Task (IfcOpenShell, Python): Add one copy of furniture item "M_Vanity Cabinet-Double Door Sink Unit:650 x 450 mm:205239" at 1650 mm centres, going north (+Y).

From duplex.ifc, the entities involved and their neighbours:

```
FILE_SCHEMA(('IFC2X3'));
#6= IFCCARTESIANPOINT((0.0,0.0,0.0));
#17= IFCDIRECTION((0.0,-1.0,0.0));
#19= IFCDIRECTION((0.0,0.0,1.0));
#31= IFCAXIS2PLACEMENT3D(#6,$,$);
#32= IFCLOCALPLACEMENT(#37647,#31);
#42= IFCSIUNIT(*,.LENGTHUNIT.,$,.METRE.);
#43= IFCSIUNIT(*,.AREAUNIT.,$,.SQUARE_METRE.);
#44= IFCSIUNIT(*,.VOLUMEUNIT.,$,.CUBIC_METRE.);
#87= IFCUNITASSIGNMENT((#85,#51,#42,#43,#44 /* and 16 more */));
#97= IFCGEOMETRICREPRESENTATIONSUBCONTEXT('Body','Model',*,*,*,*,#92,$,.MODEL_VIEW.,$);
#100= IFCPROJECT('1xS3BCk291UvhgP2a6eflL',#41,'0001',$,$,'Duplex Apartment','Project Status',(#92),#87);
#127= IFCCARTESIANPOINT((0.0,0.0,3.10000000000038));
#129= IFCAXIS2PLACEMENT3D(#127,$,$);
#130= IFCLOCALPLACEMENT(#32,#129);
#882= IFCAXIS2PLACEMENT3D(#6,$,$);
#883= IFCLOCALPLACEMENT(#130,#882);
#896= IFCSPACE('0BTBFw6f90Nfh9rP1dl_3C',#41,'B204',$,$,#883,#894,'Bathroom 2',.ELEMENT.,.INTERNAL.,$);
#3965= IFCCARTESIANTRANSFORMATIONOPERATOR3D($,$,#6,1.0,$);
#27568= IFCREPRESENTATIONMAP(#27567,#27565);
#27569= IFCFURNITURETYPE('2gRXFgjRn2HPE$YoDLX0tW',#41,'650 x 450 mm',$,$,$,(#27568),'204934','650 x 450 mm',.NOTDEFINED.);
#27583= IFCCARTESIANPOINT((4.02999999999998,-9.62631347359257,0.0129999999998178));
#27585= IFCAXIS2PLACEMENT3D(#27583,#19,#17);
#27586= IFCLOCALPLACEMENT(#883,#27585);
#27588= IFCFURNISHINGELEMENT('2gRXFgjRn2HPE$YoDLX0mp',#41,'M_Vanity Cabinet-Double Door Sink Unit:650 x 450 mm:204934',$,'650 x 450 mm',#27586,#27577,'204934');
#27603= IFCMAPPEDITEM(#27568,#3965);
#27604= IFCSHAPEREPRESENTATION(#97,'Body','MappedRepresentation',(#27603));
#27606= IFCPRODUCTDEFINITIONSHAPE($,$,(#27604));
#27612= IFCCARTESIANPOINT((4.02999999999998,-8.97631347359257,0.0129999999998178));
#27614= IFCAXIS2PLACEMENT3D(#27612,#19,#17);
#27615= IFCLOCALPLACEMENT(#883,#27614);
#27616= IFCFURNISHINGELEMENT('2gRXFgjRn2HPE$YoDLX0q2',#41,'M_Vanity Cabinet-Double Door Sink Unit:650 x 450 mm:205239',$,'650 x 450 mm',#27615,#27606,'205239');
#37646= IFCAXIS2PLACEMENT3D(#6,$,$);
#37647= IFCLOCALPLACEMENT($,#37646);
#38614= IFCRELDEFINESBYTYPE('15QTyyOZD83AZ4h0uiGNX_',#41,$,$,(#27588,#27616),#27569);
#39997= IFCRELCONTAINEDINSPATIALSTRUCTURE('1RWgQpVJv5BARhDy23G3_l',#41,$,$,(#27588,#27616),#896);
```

```python
import numpy as np
import ifcopenshell
import ifcopenshell.api.geometry
import ifcopenshell.api.root
import ifcopenshell.util.element
import ifcopenshell.util.placement
import ifcopenshell.util.unit

model = ifcopenshell.open("duplex.ifc")
unit_scale = ifcopenshell.util.unit.calculate_unit_scale(model)


def reuse_history(source, copy):
    """copy_class also copies each property set's owner history, people and application; keep the originals."""
    for rel in copy.IsDefinedBy:
        if rel.is_a("IfcRelDefinesByProperties") and (history := rel.RelatingPropertyDefinition.OwnerHistory):
            rel.RelatingPropertyDefinition.OwnerHistory = source.OwnerHistory
            ifcopenshell.util.element.remove_deep2(model, history)


source = model.by_guid("2gRXFgjRn2HPE$YoDLX0q2")
base = ifcopenshell.util.placement.get_local_placement(source.ObjectPlacement)
step = np.array([0.0, 1.0, 0.0]) * 1.65 / unit_scale

for i in range(1, 2):
    copy = ifcopenshell.api.root.copy_class(model, product=source)
    copy.Representation = ifcopenshell.util.element.copy_deep(
        model, source.Representation, exclude=["IfcGeometricRepresentationContext", "IfcRepresentationMap"]
    )
    copy.Name = "M_Vanity Cabinet-Double Door Sink Unit:650 x 450 mm"
    copy.Tag = None
    reuse_history(source, copy)
    matrix = base.copy()
    matrix[:3, 3] += i * step
    print("added at", matrix[:3, 3].round(3) + 0.0)
    ifcopenshell.api.geometry.edit_object_placement(model, product=copy, matrix=matrix, is_si=False)

model.write("duplex_rev.ifc")
```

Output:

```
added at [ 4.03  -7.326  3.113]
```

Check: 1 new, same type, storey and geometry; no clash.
